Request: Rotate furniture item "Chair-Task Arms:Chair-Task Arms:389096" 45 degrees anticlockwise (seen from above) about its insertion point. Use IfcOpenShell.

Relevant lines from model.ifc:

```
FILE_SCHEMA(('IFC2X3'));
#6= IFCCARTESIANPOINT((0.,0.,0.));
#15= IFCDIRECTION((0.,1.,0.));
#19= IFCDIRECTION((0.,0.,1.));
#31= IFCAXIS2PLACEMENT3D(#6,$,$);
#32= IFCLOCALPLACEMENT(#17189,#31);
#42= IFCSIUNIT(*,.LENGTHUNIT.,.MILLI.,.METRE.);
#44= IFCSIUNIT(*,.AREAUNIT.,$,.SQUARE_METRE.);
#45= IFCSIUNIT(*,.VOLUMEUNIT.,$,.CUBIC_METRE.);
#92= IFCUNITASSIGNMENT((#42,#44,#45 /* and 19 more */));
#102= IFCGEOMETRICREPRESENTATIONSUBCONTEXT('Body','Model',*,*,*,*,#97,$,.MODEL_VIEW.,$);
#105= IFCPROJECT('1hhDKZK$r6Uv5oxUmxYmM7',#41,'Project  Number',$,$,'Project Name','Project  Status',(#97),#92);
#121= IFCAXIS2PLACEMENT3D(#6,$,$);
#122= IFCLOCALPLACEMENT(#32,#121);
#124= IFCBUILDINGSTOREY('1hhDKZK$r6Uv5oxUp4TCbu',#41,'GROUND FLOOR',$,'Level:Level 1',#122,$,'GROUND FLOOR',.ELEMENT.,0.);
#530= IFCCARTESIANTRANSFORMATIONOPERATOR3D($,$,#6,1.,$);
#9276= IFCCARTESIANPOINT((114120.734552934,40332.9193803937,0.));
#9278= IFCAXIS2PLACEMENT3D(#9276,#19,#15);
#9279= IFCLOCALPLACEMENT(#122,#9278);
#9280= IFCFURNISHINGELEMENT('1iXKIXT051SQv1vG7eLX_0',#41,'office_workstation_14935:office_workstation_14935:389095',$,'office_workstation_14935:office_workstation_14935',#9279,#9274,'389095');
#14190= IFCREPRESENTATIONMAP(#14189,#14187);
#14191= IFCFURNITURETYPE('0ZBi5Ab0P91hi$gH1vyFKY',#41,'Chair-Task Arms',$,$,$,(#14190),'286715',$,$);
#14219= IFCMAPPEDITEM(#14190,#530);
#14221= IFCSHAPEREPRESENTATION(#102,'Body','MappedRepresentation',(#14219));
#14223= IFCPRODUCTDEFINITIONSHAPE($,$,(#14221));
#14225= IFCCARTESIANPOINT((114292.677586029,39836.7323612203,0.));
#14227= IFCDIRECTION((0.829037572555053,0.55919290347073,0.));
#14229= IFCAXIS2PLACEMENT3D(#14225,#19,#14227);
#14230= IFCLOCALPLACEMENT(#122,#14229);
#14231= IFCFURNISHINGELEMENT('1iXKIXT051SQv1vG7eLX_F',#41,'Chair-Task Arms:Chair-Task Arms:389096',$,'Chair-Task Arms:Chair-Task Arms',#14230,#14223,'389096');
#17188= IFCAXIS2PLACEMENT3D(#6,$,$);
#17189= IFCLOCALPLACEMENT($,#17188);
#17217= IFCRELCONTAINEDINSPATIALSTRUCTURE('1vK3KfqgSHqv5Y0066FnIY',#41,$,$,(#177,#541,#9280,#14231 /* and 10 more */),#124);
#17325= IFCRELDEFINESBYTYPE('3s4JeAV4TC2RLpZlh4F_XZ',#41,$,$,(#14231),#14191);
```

```python
import ifcopenshell
import ifcopenshell.api.geometry
import ifcopenshell.util.placement

model = ifcopenshell.open("model.ifc")

item = model.by_guid("1iXKIXT051SQv1vG7eLX_F")
matrix = ifcopenshell.util.placement.get_local_placement(item.ObjectPlacement)
matrix = matrix @ ifcopenshell.util.placement.rotation(45, "Z")
ifcopenshell.api.geometry.edit_object_placement(model, product=item, matrix=matrix, is_si=False)

print(ifcopenshell.util.placement.get_local_placement(item.ObjectPlacement).round(3) + 0.0)

model.write("model_rev.ifc")
```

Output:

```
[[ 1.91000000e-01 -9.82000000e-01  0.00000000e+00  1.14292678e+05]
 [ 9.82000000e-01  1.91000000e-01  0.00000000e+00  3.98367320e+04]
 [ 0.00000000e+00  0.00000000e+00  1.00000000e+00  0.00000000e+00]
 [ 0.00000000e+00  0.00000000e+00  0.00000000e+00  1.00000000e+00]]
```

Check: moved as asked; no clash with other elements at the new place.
